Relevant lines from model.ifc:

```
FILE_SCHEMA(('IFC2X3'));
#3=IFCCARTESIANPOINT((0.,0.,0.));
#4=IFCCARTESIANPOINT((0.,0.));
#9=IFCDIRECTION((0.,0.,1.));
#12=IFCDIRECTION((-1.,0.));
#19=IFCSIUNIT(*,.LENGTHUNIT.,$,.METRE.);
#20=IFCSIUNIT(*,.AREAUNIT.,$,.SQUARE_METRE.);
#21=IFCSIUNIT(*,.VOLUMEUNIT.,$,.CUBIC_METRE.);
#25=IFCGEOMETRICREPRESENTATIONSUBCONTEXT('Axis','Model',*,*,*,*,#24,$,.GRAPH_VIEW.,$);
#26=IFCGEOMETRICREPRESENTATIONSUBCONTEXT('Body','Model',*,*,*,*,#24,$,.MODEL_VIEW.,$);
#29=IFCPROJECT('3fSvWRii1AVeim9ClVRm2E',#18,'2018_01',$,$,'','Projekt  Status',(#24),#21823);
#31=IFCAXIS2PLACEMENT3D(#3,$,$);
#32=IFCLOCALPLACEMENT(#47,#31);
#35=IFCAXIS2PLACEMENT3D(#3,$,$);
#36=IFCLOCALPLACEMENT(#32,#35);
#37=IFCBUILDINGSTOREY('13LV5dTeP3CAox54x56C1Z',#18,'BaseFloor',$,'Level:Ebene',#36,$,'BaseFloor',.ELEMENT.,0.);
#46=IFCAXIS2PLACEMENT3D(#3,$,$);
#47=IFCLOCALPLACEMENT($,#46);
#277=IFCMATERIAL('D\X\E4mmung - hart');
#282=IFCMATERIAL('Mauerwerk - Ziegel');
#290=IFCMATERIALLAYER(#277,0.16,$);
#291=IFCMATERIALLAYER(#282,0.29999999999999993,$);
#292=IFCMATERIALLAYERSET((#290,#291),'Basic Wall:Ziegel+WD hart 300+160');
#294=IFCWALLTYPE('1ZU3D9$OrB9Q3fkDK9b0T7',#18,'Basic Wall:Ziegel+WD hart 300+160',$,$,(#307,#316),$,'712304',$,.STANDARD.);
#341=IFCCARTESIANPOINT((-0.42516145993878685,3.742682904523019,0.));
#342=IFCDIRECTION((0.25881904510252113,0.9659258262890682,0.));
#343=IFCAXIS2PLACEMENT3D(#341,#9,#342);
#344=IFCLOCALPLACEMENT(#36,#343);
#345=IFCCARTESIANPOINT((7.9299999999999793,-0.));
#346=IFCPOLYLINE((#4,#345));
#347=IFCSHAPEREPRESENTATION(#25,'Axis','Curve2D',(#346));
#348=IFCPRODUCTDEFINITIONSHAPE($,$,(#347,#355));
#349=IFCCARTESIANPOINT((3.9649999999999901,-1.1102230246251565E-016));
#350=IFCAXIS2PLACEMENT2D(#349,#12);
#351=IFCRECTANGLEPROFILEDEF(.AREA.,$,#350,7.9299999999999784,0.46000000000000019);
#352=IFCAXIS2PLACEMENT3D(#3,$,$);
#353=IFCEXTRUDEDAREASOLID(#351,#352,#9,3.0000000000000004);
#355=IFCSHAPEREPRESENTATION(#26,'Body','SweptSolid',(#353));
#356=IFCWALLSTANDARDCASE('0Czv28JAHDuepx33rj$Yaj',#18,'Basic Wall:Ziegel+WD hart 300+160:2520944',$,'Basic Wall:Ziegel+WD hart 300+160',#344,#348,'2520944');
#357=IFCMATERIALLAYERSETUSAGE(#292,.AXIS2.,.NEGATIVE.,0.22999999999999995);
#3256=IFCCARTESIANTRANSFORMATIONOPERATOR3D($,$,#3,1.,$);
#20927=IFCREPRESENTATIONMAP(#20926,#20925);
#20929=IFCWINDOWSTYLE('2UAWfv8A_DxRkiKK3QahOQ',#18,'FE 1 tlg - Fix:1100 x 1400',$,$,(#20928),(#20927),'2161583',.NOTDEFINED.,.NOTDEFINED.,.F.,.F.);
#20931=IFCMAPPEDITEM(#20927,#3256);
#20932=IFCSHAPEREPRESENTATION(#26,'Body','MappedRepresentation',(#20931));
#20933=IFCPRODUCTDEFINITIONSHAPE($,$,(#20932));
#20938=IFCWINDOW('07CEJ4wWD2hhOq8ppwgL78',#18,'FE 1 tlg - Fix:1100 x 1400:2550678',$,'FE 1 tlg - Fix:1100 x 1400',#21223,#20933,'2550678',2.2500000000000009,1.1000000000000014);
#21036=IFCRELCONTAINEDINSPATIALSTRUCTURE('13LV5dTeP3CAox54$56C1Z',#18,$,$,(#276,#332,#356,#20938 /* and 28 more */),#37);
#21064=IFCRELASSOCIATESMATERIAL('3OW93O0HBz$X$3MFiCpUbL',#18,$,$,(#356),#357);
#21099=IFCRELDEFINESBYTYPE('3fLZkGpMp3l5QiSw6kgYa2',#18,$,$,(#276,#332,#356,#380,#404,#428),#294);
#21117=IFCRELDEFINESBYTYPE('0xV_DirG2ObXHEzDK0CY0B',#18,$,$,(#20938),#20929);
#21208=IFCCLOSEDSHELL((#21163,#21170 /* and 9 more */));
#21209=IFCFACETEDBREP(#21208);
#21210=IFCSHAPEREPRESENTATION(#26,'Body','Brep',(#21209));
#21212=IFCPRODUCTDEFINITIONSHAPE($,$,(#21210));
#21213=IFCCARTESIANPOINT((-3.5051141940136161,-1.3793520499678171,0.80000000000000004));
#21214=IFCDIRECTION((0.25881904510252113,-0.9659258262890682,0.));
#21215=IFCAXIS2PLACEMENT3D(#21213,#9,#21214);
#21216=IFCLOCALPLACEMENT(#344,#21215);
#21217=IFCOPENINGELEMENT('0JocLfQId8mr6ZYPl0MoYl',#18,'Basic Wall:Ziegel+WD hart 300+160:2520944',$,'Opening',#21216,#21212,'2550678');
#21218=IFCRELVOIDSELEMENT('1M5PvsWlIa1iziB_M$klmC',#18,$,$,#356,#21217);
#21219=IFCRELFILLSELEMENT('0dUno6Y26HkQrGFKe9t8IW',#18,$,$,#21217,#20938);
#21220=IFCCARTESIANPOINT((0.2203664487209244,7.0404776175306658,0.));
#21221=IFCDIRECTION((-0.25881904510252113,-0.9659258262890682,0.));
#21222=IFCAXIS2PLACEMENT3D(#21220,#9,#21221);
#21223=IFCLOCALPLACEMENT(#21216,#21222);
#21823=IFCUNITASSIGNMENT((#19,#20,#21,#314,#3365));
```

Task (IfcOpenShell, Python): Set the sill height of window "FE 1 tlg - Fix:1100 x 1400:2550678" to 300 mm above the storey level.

```python
import numpy as np
import ifcopenshell
import ifcopenshell.api.geometry
import ifcopenshell.geom
import ifcopenshell.util.element
import ifcopenshell.util.placement
import ifcopenshell.util.shape
import ifcopenshell.util.unit

model = ifcopenshell.open("model.ifc")
unit_scale = ifcopenshell.util.unit.calculate_unit_scale(model)

window = model.by_guid("07CEJ4wWD2hhOq8ppwgL78")
opening = window.FillsVoids[0].RelatingOpeningElement
storey = ifcopenshell.util.element.get_container(window, ifc_class="IfcBuildingStorey")
level = ifcopenshell.util.placement.get_local_placement(storey.ObjectPlacement)[2, 3]

# The opening's origin need not be at the sill, so measure its lowest point.
shape = ifcopenshell.geom.create_shape(ifcopenshell.geom.settings(), opening)
bottom = ifcopenshell.util.shape.get_shape_bottom_elevation(shape, shape.geometry) / unit_scale
dz = level + 0.3 / unit_scale - bottom

shift = np.array([0.0, 0.0, dz])
# The window is placed relative to its opening, so it follows when the opening moves.
matrix = ifcopenshell.util.placement.get_local_placement(opening.ObjectPlacement)
matrix[:3, 3] += shift
ifcopenshell.api.geometry.edit_object_placement(
    model, product=opening, matrix=matrix, is_si=False, should_transform_children=True
)

print(f"moved by {dz * unit_scale:+.3f} m")

model.write("model_updated.ifc")
```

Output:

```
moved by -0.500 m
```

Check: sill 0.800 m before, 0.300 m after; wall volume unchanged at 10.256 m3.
